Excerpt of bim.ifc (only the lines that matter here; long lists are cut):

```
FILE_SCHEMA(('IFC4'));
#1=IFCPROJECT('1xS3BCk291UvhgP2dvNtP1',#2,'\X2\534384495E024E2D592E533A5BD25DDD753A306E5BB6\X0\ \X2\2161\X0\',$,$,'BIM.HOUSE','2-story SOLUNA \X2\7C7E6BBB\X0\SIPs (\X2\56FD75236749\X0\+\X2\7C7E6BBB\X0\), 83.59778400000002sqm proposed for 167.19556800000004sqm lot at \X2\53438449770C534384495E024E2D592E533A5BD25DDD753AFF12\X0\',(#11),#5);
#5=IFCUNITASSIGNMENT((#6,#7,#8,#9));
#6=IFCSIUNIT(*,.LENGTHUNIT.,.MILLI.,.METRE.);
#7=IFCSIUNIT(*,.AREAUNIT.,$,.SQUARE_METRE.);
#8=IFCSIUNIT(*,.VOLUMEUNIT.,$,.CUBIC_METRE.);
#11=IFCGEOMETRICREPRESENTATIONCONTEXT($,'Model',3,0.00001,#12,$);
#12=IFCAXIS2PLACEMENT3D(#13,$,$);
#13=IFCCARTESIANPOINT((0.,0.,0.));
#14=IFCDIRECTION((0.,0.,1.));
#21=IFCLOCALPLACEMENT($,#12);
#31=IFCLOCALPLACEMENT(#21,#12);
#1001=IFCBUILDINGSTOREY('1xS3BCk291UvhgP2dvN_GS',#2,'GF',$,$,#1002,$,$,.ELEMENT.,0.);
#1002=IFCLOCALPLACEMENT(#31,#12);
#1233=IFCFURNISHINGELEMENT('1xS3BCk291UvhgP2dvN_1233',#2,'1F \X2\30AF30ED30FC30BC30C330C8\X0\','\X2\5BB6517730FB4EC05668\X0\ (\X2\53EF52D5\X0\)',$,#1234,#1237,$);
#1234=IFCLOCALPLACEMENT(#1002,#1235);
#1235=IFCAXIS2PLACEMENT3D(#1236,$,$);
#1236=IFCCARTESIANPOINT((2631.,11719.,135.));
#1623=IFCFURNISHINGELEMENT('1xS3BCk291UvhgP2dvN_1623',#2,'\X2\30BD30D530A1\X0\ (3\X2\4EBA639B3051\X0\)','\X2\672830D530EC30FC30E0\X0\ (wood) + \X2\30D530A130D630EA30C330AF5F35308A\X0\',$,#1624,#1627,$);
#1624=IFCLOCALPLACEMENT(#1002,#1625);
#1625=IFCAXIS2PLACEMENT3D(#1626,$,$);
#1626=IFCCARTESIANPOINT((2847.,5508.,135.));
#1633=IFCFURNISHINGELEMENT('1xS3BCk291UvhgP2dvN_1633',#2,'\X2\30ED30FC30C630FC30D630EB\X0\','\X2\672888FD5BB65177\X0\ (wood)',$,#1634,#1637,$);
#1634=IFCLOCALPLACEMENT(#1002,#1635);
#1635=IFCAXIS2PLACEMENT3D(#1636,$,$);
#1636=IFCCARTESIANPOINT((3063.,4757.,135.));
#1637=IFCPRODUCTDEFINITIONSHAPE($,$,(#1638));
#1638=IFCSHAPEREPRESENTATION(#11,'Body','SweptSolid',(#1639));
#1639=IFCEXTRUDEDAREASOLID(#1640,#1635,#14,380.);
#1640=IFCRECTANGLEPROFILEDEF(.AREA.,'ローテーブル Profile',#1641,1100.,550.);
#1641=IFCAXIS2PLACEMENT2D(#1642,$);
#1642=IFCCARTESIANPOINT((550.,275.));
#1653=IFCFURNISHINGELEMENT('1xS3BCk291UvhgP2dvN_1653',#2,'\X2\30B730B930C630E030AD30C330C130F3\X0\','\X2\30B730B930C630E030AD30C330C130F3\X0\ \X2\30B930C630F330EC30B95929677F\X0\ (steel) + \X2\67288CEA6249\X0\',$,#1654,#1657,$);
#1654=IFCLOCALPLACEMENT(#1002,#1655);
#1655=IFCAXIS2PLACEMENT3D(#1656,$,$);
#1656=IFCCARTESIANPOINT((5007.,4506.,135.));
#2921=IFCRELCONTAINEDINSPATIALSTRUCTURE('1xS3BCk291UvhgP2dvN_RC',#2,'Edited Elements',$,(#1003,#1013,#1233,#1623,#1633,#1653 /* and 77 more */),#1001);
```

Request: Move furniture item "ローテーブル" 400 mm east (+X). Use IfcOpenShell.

```python
import ifcopenshell
import ifcopenshell.api.geometry
import ifcopenshell.util.placement

model = ifcopenshell.open("bim.ifc")

item = model.by_id(1633)
matrix = ifcopenshell.util.placement.get_local_placement(item.ObjectPlacement)
matrix[0, 3] += 400.0
ifcopenshell.api.geometry.edit_object_placement(model, product=item, matrix=matrix, is_si=False)

print(ifcopenshell.util.placement.get_local_placement(item.ObjectPlacement).round(3) + 0.0)

model.write("bim_edited.ifc")
```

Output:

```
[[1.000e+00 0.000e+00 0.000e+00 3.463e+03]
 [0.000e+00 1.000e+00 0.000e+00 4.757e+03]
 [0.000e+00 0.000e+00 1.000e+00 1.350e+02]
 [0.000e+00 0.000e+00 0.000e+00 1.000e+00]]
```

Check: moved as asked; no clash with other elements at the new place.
